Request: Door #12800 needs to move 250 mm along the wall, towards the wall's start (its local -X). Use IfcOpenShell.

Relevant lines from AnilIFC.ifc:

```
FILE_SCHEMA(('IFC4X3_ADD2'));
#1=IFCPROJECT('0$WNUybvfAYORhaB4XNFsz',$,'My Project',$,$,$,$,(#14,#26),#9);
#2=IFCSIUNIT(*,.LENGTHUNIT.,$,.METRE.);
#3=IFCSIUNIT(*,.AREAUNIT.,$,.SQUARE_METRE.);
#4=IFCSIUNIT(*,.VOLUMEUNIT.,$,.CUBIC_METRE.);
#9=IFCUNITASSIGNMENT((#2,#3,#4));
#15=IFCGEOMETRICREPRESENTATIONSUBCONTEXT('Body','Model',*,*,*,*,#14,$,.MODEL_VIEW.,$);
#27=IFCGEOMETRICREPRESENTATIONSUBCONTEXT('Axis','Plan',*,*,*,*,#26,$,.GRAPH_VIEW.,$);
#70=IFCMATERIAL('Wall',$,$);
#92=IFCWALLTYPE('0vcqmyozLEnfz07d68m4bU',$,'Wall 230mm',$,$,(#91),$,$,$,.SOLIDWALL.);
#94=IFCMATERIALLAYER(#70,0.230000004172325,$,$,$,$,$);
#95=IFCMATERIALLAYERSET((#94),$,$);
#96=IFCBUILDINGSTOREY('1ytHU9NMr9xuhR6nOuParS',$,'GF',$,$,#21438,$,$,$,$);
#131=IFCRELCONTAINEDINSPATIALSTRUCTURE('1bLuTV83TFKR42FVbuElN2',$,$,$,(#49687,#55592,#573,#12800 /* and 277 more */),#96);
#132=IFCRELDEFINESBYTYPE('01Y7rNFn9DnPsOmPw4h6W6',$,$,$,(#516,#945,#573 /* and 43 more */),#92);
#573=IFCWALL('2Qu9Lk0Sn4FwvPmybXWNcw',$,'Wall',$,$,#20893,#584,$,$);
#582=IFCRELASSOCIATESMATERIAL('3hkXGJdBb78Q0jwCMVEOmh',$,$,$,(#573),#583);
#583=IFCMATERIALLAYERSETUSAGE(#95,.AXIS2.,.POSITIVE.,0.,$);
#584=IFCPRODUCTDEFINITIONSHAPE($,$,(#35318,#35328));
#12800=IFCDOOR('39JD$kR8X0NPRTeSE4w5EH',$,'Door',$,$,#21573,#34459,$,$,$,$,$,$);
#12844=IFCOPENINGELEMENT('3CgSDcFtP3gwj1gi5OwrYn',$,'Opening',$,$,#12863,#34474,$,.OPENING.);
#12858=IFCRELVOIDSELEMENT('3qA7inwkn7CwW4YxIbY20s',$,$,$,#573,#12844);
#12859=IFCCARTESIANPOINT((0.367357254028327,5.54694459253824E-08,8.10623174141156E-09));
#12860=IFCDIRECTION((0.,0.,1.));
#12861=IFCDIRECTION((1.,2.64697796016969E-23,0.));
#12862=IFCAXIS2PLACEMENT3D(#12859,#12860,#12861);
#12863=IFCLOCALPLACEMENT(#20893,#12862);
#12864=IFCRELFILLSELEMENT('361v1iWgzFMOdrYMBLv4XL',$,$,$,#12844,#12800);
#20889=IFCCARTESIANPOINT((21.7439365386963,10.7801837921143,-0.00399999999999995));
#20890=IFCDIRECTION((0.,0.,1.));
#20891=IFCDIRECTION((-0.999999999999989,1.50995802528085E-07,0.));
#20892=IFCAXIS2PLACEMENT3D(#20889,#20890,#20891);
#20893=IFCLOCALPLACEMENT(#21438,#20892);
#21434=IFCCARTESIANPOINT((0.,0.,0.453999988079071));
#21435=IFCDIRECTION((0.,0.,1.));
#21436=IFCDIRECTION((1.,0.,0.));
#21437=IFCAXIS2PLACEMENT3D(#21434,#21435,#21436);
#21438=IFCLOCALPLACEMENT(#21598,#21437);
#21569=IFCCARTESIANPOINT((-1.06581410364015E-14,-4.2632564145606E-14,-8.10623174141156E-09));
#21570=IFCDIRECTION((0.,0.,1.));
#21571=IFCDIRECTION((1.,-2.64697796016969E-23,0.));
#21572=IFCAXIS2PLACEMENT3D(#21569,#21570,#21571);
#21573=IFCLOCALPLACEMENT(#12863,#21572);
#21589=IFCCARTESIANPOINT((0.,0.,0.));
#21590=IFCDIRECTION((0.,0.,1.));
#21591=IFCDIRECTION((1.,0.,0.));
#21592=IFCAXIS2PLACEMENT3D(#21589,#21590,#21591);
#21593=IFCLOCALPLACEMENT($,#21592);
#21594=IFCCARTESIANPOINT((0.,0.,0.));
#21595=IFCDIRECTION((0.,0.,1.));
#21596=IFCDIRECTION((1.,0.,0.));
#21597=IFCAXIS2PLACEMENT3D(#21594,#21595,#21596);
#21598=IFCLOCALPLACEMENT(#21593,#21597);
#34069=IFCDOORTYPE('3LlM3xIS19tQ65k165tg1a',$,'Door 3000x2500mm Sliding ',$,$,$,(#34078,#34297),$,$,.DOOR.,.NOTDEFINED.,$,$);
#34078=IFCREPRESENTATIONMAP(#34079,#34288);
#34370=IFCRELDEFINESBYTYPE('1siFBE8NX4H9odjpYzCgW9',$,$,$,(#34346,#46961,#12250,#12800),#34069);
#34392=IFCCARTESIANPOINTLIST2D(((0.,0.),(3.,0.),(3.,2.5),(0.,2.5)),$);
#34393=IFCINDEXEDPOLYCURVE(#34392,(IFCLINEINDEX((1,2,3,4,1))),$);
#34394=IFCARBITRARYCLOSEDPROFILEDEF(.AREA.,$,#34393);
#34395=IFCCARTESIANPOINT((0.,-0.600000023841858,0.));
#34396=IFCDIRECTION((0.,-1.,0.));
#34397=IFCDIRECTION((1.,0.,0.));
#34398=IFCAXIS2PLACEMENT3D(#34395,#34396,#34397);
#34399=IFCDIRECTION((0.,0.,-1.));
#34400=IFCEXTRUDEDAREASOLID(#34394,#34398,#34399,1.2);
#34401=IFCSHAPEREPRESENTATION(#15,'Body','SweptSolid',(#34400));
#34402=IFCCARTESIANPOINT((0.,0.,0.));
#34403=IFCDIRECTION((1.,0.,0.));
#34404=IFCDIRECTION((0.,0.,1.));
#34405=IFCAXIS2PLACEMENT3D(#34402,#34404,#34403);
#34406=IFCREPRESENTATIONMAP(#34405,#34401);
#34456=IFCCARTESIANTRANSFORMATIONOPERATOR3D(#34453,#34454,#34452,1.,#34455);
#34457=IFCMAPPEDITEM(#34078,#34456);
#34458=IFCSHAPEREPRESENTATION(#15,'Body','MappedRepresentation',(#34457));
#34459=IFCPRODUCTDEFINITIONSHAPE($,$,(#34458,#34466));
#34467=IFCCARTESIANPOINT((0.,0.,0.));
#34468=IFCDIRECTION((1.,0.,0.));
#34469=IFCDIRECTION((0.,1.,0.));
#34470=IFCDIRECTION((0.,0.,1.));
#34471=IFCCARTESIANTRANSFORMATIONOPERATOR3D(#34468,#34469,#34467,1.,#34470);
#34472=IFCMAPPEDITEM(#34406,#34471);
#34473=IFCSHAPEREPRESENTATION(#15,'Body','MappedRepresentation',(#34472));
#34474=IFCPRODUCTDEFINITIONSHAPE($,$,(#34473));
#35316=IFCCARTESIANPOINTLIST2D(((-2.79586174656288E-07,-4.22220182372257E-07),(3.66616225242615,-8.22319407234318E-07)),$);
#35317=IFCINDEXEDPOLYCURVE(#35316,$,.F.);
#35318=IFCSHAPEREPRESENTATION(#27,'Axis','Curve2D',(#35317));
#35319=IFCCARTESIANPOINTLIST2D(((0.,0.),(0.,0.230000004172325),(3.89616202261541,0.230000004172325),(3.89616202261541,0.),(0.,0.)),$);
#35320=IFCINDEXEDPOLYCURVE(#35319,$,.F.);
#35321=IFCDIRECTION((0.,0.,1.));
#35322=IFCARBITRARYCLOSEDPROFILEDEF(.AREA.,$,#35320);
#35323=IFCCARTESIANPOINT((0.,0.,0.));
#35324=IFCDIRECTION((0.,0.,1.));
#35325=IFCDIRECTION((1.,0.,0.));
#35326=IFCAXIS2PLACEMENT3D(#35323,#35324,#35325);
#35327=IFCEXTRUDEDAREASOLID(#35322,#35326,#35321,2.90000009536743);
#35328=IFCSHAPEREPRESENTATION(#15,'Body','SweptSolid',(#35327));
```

```python
import ifcopenshell
import ifcopenshell.api.geometry
import ifcopenshell.util.placement

model = ifcopenshell.open("AnilIFC.ifc")

door = model.by_guid("39JD$kR8X0NPRTeSE4w5EH")
opening = door.FillsVoids[0].RelatingOpeningElement
wall = opening.VoidsElements[0].RelatingBuildingElement

wall_matrix = ifcopenshell.util.placement.get_local_placement(wall.ObjectPlacement)
shift = wall_matrix[:3, 0] * -0.25
before = ifcopenshell.util.placement.get_local_placement(door.ObjectPlacement)[:3, 3].copy()

# The door is placed relative to its opening, so it follows when the opening moves.
matrix = ifcopenshell.util.placement.get_local_placement(opening.ObjectPlacement)
matrix[:3, 3] += shift
ifcopenshell.api.geometry.edit_object_placement(
    model, product=opening, matrix=matrix, is_si=False, should_transform_children=True
)

after = ifcopenshell.util.placement.get_local_placement(door.ObjectPlacement)[:3, 3]
print("door moved by", (after - before).round(3) + 0.0)

model.write("AnilIFC_rev.ifc")
```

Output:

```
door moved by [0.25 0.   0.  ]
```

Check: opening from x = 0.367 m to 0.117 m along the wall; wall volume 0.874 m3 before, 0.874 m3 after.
